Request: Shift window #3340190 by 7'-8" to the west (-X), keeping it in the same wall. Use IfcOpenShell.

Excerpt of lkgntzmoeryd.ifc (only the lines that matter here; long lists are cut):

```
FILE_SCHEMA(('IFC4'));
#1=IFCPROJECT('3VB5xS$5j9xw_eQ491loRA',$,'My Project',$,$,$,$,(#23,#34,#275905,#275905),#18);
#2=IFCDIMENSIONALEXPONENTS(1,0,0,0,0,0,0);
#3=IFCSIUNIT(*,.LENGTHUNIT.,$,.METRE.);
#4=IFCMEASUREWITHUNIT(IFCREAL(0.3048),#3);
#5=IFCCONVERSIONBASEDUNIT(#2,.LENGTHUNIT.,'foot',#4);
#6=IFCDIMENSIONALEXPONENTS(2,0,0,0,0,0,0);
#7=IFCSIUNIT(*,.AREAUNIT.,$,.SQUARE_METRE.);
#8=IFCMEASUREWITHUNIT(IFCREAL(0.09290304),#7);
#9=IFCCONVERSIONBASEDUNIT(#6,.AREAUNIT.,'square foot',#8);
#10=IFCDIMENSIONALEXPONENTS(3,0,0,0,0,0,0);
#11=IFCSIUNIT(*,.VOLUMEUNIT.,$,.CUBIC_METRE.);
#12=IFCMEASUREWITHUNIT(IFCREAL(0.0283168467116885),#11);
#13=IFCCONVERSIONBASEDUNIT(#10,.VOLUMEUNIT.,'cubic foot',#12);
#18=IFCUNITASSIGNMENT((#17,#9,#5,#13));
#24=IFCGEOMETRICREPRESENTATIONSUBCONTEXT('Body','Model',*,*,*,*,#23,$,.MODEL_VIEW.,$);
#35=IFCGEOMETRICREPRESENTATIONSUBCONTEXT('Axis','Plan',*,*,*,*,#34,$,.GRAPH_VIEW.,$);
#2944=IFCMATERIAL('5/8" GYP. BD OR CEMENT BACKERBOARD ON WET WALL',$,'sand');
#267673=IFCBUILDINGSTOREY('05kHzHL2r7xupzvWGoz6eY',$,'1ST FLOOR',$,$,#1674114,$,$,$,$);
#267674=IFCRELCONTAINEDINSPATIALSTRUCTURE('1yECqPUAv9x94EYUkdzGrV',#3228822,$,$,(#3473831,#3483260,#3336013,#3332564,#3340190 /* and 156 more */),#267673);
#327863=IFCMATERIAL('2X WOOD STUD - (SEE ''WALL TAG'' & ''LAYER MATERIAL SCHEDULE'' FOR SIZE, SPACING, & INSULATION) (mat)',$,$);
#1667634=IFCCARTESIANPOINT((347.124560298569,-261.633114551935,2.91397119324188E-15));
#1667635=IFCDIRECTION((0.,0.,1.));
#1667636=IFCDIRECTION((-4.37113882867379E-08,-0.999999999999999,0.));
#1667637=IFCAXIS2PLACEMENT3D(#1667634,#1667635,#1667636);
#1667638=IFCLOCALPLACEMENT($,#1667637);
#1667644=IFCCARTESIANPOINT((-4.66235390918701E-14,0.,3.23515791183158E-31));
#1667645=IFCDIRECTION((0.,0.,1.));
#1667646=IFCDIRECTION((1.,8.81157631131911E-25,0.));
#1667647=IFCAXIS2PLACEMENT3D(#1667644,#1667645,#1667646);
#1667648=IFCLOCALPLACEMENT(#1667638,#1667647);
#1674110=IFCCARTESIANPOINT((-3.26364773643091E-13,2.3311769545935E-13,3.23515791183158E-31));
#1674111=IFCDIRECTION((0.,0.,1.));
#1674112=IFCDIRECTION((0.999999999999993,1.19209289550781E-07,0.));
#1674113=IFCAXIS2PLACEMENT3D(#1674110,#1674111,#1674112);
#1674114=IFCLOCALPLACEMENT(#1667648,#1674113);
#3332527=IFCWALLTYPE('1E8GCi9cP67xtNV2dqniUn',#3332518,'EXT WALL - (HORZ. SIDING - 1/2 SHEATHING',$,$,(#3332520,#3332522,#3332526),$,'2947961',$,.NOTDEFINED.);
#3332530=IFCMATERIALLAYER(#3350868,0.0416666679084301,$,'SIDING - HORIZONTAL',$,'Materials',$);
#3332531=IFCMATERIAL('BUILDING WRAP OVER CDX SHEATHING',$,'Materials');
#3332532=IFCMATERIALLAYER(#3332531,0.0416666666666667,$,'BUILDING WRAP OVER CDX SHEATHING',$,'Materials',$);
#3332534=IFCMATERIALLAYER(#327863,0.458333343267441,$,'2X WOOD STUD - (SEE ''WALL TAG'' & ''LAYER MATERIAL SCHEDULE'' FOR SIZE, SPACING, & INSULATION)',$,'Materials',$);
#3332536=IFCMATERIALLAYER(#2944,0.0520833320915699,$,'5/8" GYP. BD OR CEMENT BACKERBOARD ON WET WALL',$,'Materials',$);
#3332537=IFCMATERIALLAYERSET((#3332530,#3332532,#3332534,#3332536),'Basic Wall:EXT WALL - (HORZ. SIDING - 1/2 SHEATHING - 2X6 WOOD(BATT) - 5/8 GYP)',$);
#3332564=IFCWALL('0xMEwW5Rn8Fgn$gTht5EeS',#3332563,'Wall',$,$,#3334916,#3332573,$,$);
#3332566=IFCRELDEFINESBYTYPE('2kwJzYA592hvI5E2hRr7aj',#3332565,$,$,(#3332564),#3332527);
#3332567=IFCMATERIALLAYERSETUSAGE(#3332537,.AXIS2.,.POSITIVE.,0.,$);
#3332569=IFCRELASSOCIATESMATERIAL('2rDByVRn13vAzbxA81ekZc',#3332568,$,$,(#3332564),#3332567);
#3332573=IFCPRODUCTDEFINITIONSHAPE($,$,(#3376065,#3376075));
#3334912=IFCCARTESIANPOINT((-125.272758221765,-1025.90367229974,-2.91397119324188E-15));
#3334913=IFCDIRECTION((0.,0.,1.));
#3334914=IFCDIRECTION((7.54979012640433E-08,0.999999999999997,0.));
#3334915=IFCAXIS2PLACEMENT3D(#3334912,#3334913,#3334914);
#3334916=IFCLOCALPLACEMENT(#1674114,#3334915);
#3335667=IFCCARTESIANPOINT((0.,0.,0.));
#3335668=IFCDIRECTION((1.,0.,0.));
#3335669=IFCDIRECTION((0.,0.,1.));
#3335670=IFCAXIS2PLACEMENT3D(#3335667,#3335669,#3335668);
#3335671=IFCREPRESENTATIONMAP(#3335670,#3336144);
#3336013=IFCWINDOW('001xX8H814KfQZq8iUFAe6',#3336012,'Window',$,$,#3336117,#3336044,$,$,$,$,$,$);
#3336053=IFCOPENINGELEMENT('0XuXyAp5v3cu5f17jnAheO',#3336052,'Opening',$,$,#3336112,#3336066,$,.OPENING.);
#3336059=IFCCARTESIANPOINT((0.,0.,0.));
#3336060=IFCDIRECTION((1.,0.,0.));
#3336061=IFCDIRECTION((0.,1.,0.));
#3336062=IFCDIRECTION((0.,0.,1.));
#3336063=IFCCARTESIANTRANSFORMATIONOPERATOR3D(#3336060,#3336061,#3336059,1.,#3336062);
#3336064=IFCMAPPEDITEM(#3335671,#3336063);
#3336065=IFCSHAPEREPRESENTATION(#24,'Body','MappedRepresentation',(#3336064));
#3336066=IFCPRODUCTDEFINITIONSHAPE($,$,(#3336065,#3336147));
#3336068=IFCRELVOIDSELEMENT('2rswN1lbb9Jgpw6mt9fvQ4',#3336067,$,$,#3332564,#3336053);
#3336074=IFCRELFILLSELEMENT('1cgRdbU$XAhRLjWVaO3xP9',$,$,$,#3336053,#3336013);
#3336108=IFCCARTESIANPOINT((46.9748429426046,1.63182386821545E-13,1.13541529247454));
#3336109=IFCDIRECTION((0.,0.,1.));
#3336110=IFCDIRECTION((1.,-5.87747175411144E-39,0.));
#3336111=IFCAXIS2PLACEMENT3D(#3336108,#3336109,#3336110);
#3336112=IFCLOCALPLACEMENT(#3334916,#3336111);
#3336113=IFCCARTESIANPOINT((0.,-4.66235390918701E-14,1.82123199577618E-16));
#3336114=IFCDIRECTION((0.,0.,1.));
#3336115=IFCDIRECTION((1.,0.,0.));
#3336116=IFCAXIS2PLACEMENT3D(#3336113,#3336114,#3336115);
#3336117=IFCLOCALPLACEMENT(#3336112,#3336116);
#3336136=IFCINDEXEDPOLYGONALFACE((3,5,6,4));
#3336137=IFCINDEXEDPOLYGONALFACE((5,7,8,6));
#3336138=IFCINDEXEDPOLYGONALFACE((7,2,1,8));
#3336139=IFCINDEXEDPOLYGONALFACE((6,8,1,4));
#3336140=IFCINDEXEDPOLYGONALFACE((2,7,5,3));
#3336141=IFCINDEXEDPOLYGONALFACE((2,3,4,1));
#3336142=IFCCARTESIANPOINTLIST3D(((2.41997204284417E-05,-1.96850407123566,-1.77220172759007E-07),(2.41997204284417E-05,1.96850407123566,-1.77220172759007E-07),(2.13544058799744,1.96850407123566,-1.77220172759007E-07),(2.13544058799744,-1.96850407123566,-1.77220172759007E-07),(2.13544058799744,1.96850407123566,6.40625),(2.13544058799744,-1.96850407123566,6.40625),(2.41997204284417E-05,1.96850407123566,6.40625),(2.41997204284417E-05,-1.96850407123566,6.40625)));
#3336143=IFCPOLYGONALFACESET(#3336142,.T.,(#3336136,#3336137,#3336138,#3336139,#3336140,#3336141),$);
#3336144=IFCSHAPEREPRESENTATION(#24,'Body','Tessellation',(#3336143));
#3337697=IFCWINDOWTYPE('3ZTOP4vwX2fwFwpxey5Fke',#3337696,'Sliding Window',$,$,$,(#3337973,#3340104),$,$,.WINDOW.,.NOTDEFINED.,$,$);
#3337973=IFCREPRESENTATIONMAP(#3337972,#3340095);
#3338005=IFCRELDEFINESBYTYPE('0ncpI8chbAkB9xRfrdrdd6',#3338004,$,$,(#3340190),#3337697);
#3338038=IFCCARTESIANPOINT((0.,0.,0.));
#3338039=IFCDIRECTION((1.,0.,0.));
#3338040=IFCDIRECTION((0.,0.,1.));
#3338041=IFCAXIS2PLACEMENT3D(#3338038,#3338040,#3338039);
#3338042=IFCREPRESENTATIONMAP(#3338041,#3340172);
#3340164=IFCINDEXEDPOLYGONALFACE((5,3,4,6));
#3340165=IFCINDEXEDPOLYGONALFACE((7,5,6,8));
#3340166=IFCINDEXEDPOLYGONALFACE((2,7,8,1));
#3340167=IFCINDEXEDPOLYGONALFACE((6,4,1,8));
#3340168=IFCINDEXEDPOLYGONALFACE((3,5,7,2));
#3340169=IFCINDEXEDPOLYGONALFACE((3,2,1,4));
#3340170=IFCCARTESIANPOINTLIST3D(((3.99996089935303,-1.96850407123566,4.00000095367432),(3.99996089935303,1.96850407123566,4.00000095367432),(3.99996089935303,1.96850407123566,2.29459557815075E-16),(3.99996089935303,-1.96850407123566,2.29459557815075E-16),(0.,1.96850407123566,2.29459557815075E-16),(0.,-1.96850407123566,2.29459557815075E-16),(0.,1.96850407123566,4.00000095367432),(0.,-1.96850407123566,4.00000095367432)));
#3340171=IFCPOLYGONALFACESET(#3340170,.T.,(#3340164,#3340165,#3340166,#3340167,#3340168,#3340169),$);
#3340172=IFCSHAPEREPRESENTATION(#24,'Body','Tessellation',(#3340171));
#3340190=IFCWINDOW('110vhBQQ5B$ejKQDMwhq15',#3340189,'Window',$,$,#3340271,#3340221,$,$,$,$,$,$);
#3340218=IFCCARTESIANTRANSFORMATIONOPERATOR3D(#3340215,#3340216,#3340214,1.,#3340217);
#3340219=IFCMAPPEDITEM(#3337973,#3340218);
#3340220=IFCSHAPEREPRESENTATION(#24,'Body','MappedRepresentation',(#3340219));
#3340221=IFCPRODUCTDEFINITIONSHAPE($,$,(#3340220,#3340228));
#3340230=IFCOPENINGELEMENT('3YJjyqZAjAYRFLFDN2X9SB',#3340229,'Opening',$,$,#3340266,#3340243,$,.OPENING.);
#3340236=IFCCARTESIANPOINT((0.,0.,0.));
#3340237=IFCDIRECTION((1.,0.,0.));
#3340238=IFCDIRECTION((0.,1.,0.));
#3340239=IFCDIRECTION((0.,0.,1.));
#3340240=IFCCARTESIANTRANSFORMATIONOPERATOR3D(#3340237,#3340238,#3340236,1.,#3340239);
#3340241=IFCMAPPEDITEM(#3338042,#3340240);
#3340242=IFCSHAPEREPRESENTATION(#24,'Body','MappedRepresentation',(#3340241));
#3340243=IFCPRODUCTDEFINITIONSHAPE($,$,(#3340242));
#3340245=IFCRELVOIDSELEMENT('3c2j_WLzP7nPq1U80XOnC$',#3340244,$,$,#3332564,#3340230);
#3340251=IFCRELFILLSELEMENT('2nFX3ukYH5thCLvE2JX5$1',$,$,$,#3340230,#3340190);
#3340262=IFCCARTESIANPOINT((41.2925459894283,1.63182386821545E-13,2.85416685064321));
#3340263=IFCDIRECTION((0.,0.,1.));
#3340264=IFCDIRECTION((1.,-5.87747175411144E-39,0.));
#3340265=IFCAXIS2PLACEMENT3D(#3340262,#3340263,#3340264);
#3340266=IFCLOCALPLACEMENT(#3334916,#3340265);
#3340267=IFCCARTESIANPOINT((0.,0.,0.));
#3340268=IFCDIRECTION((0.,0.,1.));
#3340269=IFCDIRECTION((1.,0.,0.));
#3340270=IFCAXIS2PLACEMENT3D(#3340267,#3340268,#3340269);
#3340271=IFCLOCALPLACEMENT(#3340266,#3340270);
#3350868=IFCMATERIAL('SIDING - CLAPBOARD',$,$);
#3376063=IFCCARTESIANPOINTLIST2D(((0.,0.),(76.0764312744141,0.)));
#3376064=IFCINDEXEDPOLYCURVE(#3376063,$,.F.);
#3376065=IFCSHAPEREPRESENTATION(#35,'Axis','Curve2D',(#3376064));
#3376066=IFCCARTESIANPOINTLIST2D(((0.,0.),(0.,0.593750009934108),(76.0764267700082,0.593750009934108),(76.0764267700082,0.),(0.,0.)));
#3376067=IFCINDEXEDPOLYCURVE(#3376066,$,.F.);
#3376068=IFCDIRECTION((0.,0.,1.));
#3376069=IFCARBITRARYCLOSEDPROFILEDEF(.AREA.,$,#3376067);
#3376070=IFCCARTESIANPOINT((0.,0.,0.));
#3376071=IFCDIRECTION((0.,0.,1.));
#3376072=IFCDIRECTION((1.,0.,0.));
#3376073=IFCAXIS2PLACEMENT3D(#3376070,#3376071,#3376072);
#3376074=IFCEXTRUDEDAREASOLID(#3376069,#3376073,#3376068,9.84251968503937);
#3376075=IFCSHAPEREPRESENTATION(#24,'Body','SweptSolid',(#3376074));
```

```python
import ifcopenshell
import ifcopenshell.api.geometry
import ifcopenshell.util.placement
import ifcopenshell.util.unit

model = ifcopenshell.open("lkgntzmoeryd.ifc")
unit_scale = ifcopenshell.util.unit.calculate_unit_scale(model)

window = model.by_guid("110vhBQQ5B$ejKQDMwhq15")
opening = window.FillsVoids[0].RelatingOpeningElement
wall = opening.VoidsElements[0].RelatingBuildingElement

wall_matrix = ifcopenshell.util.placement.get_local_placement(wall.ObjectPlacement)
shift = wall_matrix[:3, 0] * -92 * 0.0254 / unit_scale
before = ifcopenshell.util.placement.get_local_placement(window.ObjectPlacement)[:3, 3].copy()

# The window is placed relative to its opening, so it follows when the opening moves.
matrix = ifcopenshell.util.placement.get_local_placement(opening.ObjectPlacement)
matrix[:3, 3] += shift
ifcopenshell.api.geometry.edit_object_placement(
    model, product=opening, matrix=matrix, is_si=False, should_transform_children=True
)

after = ifcopenshell.util.placement.get_local_placement(window.ObjectPlacement)[:3, 3]
print("window moved by", (after - before).round(3) + 0.0)

model.write("lkgntzmoeryd_v2.ifc")
```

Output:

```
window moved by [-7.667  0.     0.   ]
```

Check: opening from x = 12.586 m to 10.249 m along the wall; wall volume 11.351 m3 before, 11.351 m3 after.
